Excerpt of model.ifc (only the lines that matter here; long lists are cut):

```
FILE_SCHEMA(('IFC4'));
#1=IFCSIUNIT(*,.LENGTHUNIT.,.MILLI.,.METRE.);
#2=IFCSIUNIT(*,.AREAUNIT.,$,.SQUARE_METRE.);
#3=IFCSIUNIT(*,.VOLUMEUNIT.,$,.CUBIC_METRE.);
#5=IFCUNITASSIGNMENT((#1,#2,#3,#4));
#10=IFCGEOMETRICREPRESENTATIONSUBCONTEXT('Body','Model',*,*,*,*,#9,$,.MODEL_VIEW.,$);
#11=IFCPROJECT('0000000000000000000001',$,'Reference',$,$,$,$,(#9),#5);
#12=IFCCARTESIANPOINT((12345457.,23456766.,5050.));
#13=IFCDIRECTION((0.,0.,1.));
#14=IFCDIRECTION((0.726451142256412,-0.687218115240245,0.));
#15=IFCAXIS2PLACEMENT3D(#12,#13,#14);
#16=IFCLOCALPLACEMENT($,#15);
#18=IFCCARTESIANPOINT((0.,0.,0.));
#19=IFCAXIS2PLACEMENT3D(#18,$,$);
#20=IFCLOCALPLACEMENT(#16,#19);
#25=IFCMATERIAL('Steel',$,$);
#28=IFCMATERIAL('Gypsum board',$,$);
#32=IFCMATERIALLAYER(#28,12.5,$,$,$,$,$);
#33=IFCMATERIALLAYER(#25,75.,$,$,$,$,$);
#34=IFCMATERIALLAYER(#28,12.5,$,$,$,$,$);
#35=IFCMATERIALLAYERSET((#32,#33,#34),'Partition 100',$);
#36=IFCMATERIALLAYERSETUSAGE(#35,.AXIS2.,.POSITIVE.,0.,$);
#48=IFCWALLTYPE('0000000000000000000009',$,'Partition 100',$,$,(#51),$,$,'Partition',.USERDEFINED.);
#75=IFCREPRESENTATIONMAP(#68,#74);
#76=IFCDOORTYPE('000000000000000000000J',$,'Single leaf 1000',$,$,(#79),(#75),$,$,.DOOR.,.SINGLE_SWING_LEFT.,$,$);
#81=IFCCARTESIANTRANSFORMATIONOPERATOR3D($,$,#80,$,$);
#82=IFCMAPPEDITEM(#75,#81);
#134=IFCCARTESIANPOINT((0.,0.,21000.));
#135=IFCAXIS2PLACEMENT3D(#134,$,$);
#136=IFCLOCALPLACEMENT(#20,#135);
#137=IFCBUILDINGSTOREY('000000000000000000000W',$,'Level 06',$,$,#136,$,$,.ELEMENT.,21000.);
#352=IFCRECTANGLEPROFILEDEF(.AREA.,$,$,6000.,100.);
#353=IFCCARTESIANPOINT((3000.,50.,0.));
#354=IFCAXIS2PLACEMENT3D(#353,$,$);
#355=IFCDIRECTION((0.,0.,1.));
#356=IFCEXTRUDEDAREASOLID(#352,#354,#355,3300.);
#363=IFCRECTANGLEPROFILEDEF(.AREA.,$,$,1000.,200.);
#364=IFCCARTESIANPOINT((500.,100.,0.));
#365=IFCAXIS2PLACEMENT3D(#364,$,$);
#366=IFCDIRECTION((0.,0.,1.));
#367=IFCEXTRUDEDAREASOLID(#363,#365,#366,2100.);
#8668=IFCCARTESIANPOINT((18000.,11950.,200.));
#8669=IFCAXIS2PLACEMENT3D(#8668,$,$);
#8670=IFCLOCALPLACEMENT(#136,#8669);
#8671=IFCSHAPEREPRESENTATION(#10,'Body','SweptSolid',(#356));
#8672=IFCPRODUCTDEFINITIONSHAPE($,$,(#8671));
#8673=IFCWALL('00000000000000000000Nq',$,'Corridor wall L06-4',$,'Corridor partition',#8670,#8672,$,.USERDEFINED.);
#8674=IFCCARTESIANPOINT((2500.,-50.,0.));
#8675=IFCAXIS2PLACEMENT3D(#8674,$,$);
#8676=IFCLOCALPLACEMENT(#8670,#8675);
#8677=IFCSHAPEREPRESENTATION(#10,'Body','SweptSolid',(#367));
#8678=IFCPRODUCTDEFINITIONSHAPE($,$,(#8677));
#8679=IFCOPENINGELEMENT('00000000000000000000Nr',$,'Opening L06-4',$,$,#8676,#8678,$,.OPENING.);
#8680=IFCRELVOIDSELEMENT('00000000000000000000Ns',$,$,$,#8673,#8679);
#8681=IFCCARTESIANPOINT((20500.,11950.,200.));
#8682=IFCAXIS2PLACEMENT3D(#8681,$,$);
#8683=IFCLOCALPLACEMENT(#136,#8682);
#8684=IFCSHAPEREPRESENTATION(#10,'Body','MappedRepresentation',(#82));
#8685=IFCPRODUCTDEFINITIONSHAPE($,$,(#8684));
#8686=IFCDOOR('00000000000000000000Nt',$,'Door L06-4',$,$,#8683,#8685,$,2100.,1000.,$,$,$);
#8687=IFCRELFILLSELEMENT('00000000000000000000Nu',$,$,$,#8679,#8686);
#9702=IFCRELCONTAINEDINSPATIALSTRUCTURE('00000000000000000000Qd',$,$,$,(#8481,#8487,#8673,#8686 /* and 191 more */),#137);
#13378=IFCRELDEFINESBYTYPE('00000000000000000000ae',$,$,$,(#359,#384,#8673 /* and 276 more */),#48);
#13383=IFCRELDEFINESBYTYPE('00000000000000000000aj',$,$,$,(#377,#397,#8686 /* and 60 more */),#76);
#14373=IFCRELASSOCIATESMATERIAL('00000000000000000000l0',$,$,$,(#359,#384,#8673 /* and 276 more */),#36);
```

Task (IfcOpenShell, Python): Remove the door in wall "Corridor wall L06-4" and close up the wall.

```python
import ifcopenshell
import ifcopenshell.api.feature
import ifcopenshell.api.root
import ifcopenshell.geom
import ifcopenshell.util.shape

model = ifcopenshell.open("model.ifc")
settings = ifcopenshell.geom.settings()


def volume(element):
    """Net volume in cubic metres, openings subtracted."""
    shape = ifcopenshell.geom.create_shape(settings, element)
    return ifcopenshell.util.shape.get_volume(shape.geometry)


door = model.by_guid("00000000000000000000Nt")
opening = door.FillsVoids[0].RelatingOpeningElement
wall = opening.VoidsElements[0].RelatingBuildingElement
before = volume(wall)

ifcopenshell.api.root.remove_product(model, product=door)
ifcopenshell.api.feature.remove_feature(model, feature=opening)

after = volume(wall)

print(f"wall volume {before:.3f} -> {after:.3f} m3")

model.write("model_updated.ifc")
```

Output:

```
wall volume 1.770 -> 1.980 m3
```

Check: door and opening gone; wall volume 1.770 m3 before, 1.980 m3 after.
